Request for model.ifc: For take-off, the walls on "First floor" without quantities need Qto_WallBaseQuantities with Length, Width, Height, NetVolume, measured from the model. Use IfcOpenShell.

First a look at what the model holds.

```python
import ifcopenshell
import ifcopenshell.util.element
import ifcopenshell.util.unit

model = ifcopenshell.open("model.ifc")
print(model.schema)
for unit_type in ("LENGTHUNIT", "AREAUNIT", "VOLUMEUNIT"):
    print(unit_type, ifcopenshell.util.unit.calculate_unit_scale(model, unit_type))
storey = next(s for s in model.by_type("IfcBuildingStorey") if s.Name == "First floor")
walls = [e for e in ifcopenshell.util.element.get_decomposition(storey) if e.is_a("IfcWall")]
for e in sorted(walls, key=lambda e: e.id()):
    print(e.id(), e.is_a(), e.Name, list(ifcopenshell.util.element.get_psets(e, qtos_only=True)), sep=" | ")
```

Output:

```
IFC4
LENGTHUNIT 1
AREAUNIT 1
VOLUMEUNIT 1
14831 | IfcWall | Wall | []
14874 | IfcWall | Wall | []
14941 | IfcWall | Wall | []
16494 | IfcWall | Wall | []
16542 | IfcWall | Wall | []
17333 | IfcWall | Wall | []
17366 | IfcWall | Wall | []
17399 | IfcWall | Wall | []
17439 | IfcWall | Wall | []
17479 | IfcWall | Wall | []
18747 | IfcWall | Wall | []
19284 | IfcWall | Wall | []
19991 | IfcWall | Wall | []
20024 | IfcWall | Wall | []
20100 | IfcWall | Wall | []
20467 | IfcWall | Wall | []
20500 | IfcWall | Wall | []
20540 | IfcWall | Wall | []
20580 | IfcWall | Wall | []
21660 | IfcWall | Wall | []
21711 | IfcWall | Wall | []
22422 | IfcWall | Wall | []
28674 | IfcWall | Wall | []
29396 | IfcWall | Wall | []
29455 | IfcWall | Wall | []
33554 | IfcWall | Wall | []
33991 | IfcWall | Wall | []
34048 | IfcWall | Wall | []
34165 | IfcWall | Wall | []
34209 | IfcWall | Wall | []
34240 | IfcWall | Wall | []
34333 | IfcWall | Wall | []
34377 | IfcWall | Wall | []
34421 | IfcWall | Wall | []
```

```python
import ifcopenshell
import ifcopenshell.api.pset
import ifcopenshell.geom
import ifcopenshell.util.element
import ifcopenshell.util.shape
import ifcopenshell.util.unit

model = ifcopenshell.open("model.ifc")
unit_scale = ifcopenshell.util.unit.calculate_unit_scale(model)
volume_scale = ifcopenshell.util.unit.calculate_unit_scale(model, "VOLUMEUNIT")
settings = ifcopenshell.geom.settings()

storey = next(s for s in model.by_type("IfcBuildingStorey") if s.Name == "First floor")
walls = [e for e in ifcopenshell.util.element.get_decomposition(storey) if e.is_a("IfcWall")]

for e in sorted(walls, key=lambda e: e.id()):
    if ifcopenshell.util.element.get_psets(e, qtos_only=True, should_inherit=False):
        continue
    # Geometry comes back in metres, in the element's own axes.
    shape = ifcopenshell.geom.create_shape(settings, e)
    values = {
        "Length": ifcopenshell.util.shape.get_x(shape.geometry) / unit_scale,
        "Width": ifcopenshell.util.shape.get_y(shape.geometry) / unit_scale,
        "Height": ifcopenshell.util.shape.get_z(shape.geometry) / unit_scale,
        "NetVolume": ifcopenshell.util.shape.get_volume(shape.geometry) / volume_scale,
    }
    qto = ifcopenshell.api.pset.add_qto(model, product=e, name="Qto_WallBaseQuantities")
    ifcopenshell.api.pset.edit_qto(model, qto=qto, properties=values)
    print(e.id(), {k: round(v, 3) for k, v in values.items()})

model.write("model-out.ifc")
```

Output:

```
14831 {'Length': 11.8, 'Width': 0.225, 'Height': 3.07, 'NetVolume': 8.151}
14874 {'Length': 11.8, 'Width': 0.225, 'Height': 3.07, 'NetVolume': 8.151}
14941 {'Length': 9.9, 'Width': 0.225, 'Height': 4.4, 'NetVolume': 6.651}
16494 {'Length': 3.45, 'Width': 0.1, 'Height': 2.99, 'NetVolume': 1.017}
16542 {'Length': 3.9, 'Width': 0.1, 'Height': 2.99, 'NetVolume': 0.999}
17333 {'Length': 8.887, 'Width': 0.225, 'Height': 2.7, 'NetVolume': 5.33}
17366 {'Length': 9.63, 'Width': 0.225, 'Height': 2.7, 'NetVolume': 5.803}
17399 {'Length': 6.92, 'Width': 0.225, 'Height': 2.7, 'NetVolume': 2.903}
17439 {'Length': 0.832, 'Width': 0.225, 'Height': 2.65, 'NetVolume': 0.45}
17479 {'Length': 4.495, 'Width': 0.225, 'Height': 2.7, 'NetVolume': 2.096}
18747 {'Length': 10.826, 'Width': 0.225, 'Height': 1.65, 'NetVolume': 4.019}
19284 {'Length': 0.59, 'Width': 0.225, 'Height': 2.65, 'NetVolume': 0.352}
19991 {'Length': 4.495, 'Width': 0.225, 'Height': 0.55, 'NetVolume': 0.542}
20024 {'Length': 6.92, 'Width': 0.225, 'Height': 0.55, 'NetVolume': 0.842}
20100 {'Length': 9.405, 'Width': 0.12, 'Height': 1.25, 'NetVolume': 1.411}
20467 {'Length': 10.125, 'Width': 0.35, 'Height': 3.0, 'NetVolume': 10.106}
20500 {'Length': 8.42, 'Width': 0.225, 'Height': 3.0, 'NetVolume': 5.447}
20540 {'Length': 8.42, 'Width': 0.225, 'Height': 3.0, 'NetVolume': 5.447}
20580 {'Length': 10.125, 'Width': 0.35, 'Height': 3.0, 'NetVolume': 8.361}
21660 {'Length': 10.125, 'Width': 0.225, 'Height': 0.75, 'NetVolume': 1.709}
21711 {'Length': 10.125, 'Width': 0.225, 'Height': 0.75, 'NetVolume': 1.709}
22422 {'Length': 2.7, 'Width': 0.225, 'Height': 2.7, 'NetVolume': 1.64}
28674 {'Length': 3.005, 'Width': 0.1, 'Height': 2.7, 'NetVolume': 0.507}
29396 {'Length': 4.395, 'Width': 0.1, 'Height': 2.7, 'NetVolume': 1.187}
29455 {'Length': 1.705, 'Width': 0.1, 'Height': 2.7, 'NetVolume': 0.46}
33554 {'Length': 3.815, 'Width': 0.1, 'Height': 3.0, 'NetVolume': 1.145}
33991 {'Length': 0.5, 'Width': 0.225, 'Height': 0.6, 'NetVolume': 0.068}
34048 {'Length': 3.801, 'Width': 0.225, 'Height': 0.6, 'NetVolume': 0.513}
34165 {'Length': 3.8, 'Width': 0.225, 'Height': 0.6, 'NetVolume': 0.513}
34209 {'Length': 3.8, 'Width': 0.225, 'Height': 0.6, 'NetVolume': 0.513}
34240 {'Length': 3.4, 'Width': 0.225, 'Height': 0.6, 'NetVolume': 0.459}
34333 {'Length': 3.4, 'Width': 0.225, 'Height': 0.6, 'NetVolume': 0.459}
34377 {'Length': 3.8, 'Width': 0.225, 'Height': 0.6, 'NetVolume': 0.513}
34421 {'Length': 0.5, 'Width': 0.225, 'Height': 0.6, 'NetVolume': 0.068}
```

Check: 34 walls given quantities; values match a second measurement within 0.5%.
